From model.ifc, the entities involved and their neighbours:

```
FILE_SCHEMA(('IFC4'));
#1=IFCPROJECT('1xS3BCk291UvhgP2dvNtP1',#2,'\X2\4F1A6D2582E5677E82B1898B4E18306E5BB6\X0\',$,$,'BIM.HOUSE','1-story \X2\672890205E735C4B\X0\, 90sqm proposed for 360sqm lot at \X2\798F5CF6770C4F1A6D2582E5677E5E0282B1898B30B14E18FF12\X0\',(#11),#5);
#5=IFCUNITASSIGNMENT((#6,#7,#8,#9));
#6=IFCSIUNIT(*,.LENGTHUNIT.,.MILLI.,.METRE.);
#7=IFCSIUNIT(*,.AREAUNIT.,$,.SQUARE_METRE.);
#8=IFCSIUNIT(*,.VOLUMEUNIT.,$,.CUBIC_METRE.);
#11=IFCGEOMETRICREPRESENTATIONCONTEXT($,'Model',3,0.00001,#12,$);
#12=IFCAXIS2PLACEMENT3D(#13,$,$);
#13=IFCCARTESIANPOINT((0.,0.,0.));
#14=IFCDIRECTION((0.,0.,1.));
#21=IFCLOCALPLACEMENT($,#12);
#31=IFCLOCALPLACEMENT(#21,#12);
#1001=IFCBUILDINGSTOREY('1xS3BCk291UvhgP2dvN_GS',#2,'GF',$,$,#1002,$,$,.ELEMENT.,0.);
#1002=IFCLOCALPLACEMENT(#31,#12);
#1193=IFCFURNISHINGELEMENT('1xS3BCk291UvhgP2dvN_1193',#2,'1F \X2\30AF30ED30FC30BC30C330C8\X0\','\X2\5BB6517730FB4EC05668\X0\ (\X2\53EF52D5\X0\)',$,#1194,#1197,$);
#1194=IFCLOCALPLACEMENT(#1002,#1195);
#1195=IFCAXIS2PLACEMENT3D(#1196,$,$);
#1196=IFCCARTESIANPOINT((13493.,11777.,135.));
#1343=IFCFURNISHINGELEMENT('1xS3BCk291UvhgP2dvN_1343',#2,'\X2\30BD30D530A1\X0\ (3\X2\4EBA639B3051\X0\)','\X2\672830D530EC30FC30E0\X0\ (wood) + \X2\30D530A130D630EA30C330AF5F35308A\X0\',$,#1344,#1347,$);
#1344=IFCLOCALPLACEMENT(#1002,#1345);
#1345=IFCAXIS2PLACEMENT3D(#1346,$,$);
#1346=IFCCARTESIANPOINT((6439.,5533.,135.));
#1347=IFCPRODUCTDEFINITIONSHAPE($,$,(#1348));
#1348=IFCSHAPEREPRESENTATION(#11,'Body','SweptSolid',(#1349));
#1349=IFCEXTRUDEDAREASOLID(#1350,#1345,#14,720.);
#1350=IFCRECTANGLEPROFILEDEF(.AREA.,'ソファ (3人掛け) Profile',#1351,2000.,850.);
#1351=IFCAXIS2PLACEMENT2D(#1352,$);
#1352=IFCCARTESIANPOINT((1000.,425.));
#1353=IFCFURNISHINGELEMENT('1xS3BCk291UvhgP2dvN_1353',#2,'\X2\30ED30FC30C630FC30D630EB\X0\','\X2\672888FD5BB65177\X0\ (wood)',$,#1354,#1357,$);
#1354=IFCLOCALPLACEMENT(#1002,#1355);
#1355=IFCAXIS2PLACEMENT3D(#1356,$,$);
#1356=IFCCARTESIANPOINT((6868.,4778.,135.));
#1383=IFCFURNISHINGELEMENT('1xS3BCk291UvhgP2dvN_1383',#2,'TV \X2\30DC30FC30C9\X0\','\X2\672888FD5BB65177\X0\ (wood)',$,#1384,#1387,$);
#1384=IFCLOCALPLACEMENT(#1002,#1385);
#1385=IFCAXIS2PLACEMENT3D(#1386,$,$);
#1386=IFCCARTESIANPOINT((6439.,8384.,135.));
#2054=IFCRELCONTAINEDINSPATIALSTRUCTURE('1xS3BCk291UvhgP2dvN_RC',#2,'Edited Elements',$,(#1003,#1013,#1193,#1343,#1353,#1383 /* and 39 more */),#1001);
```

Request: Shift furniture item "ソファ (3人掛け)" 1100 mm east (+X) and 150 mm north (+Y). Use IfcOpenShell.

```python
import ifcopenshell
import ifcopenshell.api.geometry
import ifcopenshell.util.placement

model = ifcopenshell.open("model.ifc")

item = model.by_id(1343)
matrix = ifcopenshell.util.placement.get_local_placement(item.ObjectPlacement)
matrix[0, 3] += 1100.0
matrix[1, 3] += 150.0
ifcopenshell.api.geometry.edit_object_placement(model, product=item, matrix=matrix, is_si=False)

print(ifcopenshell.util.placement.get_local_placement(item.ObjectPlacement).round(3) + 0.0)

model.write("model_edited.ifc")
```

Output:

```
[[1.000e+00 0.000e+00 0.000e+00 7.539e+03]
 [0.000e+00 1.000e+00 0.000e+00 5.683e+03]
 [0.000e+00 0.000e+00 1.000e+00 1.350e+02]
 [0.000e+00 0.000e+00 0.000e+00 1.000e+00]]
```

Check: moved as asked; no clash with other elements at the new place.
